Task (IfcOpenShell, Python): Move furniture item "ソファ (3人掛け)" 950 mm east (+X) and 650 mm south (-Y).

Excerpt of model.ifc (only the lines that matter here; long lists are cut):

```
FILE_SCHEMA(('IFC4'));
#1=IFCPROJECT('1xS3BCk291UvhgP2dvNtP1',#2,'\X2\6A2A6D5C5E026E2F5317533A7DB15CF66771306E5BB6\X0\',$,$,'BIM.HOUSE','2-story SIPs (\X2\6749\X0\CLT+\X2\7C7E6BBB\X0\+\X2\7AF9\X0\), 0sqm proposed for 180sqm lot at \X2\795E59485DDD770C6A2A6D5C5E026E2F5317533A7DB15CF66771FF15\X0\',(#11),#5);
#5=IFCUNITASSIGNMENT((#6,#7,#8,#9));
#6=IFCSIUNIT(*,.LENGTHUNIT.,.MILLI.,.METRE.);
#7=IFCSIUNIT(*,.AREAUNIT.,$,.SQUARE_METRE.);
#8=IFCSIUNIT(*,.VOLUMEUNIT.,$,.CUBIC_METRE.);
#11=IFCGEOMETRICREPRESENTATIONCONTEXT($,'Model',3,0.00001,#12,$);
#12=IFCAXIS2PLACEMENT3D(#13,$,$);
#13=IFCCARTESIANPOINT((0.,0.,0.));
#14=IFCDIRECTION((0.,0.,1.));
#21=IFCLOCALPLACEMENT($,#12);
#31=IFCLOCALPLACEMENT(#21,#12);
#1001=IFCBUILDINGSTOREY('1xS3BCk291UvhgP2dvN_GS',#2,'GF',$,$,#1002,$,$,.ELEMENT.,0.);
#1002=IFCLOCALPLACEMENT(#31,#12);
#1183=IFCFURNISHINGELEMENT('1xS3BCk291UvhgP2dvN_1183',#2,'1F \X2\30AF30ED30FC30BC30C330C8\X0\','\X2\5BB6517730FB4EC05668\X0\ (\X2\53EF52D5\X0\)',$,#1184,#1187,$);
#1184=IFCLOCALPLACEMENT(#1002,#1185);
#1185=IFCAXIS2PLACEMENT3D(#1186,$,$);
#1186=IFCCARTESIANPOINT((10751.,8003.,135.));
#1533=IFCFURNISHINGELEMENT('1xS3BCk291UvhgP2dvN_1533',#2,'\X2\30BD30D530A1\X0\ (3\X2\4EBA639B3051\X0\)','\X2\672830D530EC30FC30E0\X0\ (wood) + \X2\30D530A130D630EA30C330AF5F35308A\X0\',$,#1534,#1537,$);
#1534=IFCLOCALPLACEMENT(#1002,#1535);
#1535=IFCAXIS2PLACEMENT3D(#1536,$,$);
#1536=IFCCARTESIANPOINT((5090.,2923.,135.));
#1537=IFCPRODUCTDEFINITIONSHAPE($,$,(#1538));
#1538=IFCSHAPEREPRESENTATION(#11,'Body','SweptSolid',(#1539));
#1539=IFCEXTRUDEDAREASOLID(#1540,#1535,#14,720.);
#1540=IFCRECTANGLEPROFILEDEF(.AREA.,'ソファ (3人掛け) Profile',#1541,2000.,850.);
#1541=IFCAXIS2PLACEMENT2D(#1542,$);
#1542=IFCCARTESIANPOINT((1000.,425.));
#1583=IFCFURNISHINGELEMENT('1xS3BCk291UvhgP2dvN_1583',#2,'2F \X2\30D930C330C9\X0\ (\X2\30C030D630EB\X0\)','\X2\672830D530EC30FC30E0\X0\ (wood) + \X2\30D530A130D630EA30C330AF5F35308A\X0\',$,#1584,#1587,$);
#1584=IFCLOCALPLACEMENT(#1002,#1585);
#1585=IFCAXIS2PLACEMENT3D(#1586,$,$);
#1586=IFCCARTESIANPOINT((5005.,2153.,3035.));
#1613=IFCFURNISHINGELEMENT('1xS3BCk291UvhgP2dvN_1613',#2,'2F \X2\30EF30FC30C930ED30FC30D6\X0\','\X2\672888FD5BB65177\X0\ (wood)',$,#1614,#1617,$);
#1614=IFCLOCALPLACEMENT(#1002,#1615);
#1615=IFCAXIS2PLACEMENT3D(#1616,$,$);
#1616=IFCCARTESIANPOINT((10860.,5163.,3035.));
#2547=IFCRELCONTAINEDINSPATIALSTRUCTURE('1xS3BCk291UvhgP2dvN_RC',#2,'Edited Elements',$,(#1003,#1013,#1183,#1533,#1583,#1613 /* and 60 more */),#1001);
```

```python
import ifcopenshell
import ifcopenshell.api.geometry
import ifcopenshell.util.placement

model = ifcopenshell.open("model.ifc")

item = model.by_guid("1xS3BCk291UvhgP2dvN_1533")
matrix = ifcopenshell.util.placement.get_local_placement(item.ObjectPlacement)
matrix[0, 3] += 950.0
matrix[1, 3] -= 650.0
ifcopenshell.api.geometry.edit_object_placement(model, product=item, matrix=matrix, is_si=False)

print(ifcopenshell.util.placement.get_local_placement(item.ObjectPlacement).round(3) + 0.0)

model.write("model_rev.ifc")
```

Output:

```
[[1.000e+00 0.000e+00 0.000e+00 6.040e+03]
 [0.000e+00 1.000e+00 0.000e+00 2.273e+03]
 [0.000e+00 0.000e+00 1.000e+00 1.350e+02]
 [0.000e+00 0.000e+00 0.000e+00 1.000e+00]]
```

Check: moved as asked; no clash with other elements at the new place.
